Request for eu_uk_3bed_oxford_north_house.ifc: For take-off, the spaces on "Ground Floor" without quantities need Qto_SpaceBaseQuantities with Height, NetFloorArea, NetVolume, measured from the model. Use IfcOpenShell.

First a look at what the model holds.

```python
import ifcopenshell
import ifcopenshell.util.element
import ifcopenshell.util.unit

model = ifcopenshell.open("eu_uk_3bed_oxford_north_house.ifc")
print(model.schema)
for unit_type in ("LENGTHUNIT", "AREAUNIT", "VOLUMEUNIT"):
    print(unit_type, ifcopenshell.util.unit.calculate_unit_scale(model, unit_type))
storey = next(s for s in model.by_type("IfcBuildingStorey") if s.Name == "Ground Floor")
spaces = [e for e in ifcopenshell.util.element.get_decomposition(storey) if e.is_a("IfcSpace")]
for e in sorted(spaces, key=lambda e: e.id()):
    print(e.id(), e.is_a(), e.Name, list(ifcopenshell.util.element.get_psets(e, qtos_only=True)), sep=" | ")
```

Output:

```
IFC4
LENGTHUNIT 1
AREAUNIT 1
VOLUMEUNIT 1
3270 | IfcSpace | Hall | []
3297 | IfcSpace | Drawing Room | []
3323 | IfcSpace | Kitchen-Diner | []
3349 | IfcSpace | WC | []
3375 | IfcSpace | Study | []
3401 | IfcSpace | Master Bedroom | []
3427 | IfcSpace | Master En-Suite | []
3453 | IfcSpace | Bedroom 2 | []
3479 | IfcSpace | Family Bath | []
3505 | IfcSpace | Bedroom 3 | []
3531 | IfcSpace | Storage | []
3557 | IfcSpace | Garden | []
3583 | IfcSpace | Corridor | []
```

```python
import ifcopenshell
import ifcopenshell.api.pset
import ifcopenshell.geom
import ifcopenshell.util.element
import ifcopenshell.util.shape
import ifcopenshell.util.unit

model = ifcopenshell.open("eu_uk_3bed_oxford_north_house.ifc")
unit_scale = ifcopenshell.util.unit.calculate_unit_scale(model)
area_scale = ifcopenshell.util.unit.calculate_unit_scale(model, "AREAUNIT")
volume_scale = ifcopenshell.util.unit.calculate_unit_scale(model, "VOLUMEUNIT")
settings = ifcopenshell.geom.settings()

storey = next(s for s in model.by_type("IfcBuildingStorey") if s.Name == "Ground Floor")
spaces = [e for e in ifcopenshell.util.element.get_decomposition(storey) if e.is_a("IfcSpace")]

for e in sorted(spaces, key=lambda e: e.id()):
    if ifcopenshell.util.element.get_psets(e, qtos_only=True, should_inherit=False):
        continue
    # Geometry comes back in metres, in the element's own axes.
    shape = ifcopenshell.geom.create_shape(settings, e)
    values = {
        "Height": ifcopenshell.util.shape.get_z(shape.geometry) / unit_scale,
        "NetFloorArea": ifcopenshell.util.shape.get_footprint_area(shape.geometry) / area_scale,
        "NetVolume": ifcopenshell.util.shape.get_volume(shape.geometry) / volume_scale,
    }
    qto = ifcopenshell.api.pset.add_qto(model, product=e, name="Qto_SpaceBaseQuantities")
    ifcopenshell.api.pset.edit_qto(model, qto=qto, properties=values)
    print(e.id(), {k: round(v, 3) for k, v in values.items()})

model.write("eu_uk_3bed_oxford_north_house-out.ifc")
```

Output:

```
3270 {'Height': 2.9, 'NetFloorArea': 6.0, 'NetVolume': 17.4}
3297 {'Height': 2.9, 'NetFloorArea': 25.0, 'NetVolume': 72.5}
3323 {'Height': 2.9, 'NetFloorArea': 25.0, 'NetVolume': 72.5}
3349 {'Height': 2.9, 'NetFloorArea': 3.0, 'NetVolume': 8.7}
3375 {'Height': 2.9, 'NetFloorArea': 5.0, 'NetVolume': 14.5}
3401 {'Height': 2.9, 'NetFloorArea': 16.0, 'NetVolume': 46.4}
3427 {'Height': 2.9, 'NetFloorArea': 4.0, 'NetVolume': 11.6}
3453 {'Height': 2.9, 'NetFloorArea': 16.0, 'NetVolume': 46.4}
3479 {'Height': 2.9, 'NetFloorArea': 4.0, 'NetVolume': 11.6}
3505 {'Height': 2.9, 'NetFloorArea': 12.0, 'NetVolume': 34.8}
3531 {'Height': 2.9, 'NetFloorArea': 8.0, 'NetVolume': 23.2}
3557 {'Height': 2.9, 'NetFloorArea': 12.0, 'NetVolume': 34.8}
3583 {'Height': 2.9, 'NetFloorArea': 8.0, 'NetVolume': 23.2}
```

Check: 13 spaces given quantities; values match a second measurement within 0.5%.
